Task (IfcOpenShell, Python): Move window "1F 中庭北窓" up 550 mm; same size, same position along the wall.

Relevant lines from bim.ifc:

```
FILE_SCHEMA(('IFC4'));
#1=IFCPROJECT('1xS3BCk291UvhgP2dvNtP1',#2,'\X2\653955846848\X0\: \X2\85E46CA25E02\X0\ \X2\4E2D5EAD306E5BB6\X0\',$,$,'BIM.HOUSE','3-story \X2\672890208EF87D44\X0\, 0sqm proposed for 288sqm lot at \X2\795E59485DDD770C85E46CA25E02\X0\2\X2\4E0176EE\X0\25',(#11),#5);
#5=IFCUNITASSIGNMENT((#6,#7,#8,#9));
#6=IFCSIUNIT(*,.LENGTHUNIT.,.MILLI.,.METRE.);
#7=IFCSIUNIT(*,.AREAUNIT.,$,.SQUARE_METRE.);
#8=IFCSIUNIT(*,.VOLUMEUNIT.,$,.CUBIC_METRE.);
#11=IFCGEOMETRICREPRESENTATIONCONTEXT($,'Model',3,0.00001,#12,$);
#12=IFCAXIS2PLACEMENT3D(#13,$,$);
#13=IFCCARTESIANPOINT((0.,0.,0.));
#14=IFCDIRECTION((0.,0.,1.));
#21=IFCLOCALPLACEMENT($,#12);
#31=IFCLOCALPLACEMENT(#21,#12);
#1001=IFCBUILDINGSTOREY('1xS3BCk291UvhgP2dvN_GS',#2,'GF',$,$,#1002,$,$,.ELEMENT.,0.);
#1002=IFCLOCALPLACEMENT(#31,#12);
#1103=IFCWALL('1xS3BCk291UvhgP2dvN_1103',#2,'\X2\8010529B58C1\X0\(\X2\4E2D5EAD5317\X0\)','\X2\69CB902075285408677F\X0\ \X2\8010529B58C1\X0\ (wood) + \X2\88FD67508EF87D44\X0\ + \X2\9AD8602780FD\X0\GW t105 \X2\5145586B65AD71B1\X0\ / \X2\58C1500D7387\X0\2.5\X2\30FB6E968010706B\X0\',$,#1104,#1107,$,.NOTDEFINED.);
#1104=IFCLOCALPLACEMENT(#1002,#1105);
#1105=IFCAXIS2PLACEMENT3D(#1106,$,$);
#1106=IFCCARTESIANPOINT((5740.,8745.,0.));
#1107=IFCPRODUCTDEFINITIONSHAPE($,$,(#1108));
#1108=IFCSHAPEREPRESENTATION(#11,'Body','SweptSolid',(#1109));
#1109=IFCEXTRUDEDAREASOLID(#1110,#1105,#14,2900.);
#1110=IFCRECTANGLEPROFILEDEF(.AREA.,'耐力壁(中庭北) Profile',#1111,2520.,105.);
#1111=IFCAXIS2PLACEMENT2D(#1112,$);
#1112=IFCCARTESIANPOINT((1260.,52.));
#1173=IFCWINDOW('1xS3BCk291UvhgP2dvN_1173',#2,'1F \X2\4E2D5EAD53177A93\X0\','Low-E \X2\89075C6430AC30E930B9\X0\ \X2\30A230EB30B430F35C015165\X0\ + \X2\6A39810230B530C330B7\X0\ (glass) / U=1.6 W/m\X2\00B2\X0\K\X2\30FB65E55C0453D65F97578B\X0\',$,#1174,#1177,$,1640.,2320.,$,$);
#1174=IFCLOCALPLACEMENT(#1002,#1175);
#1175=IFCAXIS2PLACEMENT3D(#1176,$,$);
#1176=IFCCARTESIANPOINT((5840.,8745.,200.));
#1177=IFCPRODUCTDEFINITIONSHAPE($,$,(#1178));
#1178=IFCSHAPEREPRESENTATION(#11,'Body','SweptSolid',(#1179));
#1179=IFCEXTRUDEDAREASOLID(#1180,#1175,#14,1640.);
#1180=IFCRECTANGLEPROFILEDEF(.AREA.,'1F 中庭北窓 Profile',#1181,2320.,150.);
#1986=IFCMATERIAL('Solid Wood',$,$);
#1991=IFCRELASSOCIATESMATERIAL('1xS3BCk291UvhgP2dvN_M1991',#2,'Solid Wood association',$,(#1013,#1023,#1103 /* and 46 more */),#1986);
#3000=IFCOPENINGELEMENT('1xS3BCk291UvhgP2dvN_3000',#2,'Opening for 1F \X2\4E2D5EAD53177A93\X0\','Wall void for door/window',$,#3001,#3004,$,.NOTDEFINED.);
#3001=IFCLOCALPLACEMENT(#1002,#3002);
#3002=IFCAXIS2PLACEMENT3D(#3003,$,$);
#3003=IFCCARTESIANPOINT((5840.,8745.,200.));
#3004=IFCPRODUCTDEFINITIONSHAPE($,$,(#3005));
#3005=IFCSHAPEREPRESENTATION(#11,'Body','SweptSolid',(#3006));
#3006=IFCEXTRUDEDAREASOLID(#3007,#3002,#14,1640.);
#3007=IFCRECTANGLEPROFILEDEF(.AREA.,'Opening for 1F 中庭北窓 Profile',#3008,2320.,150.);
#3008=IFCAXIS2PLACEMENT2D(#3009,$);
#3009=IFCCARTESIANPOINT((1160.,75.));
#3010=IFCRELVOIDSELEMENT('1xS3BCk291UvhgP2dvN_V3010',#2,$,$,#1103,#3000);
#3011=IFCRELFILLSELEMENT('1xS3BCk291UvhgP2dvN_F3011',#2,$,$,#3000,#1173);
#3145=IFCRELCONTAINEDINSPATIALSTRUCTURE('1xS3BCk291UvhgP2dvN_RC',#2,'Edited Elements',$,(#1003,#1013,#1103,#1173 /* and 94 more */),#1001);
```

```python
import numpy as np
import ifcopenshell
import ifcopenshell.api.geometry
import ifcopenshell.util.placement
import ifcopenshell.util.unit

model = ifcopenshell.open("bim.ifc")
unit_scale = ifcopenshell.util.unit.calculate_unit_scale(model)

window = model.by_id(1173)
opening = window.FillsVoids[0].RelatingOpeningElement
dz = 550.0

shift = np.array([0.0, 0.0, dz])
# The window is not placed relative to its opening, so move both.
for product in (opening, window):
    matrix = ifcopenshell.util.placement.get_local_placement(product.ObjectPlacement)
    matrix[:3, 3] += shift
    ifcopenshell.api.geometry.edit_object_placement(model, product=product, matrix=matrix, is_si=False)

print(f"moved by {dz * unit_scale:+.3f} m")

model.write("bim_rev.ifc")
```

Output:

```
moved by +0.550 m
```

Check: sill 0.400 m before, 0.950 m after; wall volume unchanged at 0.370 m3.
